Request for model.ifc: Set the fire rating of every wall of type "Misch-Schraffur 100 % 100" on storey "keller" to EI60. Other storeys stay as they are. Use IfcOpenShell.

First a look at what the model holds.

```python
import ifcopenshell
import ifcopenshell.util.element

model = ifcopenshell.open("model.ifc")
print(model.schema)
storey = next(s for s in model.by_type("IfcBuildingStorey") if s.Name == "keller")
walls = [e for e in ifcopenshell.util.element.get_decomposition(storey) if e.is_a("IfcWall")]
seen = {}
for e in walls:
    element_type = ifcopenshell.util.element.get_type(e)
    key = (element_type.Name if element_type != e and element_type else None, ifcopenshell.util.element.get_pset(e, "Pset_WallCommon", "FireRating"))
    seen[key] = seen.get(key, 0) + 1
for (name, value), count in sorted(seen.items(), key=str):
    print(count, "x", name, "|", value)
```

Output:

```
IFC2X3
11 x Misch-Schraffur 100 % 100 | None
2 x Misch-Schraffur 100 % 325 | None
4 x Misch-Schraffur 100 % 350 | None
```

```python
import ifcopenshell
import ifcopenshell.api.pset
import ifcopenshell.util.element

model = ifcopenshell.open("model.ifc")

storey = next(s for s in model.by_type("IfcBuildingStorey") if s.Name == "keller")
walls = [e for e in ifcopenshell.util.element.get_decomposition(storey) if e.is_a("IfcWall")]

count = 0
for e in walls:
    element_type = ifcopenshell.util.element.get_type(e)
    if element_type in (None, e) or element_type.Name != "Misch-Schraffur 100 % 100":
        continue
    # add_pset returns the element's existing set when there is one.
    pset = ifcopenshell.api.pset.add_pset(model, product=e, name="Pset_WallCommon")
    ifcopenshell.api.pset.edit_pset(model, pset=pset, properties={"FireRating": "EI60"})
    count += 1

print(count, "walls updated")

model.write("model_rev.ifc")
```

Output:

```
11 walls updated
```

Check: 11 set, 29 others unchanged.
